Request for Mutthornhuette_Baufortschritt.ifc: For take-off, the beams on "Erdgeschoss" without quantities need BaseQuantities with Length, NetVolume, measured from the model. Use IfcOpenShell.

First a look at what the model holds.

```python
import ifcopenshell
import ifcopenshell.util.element
import ifcopenshell.util.unit

model = ifcopenshell.open("Mutthornhuette_Baufortschritt.ifc")
print(model.schema)
for unit_type in ("LENGTHUNIT", "AREAUNIT", "VOLUMEUNIT"):
    print(unit_type, ifcopenshell.util.unit.calculate_unit_scale(model, unit_type))
storey = next(s for s in model.by_type("IfcBuildingStorey") if s.Name == "Erdgeschoss")
beams = [e for e in ifcopenshell.util.element.get_decomposition(storey) if e.is_a("IfcBeam")]
for e in sorted(beams, key=lambda e: e.id()):
    print(e.id(), e.is_a(), e.Name, list(ifcopenshell.util.element.get_psets(e, qtos_only=True)), sep=" | ")
```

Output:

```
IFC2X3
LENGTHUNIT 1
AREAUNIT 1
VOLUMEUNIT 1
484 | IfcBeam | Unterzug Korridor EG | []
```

```python
import ifcopenshell
import ifcopenshell.api.pset
import ifcopenshell.geom
import ifcopenshell.util.element
import ifcopenshell.util.shape
import ifcopenshell.util.unit

model = ifcopenshell.open("Mutthornhuette_Baufortschritt.ifc")
unit_scale = ifcopenshell.util.unit.calculate_unit_scale(model)
volume_scale = ifcopenshell.util.unit.calculate_unit_scale(model, "VOLUMEUNIT")
settings = ifcopenshell.geom.settings()

storey = next(s for s in model.by_type("IfcBuildingStorey") if s.Name == "Erdgeschoss")
beams = [e for e in ifcopenshell.util.element.get_decomposition(storey) if e.is_a("IfcBeam")]

for e in sorted(beams, key=lambda e: e.id()):
    if ifcopenshell.util.element.get_psets(e, qtos_only=True, should_inherit=False):
        continue
    # Geometry comes back in metres, in the element's own axes.
    shape = ifcopenshell.geom.create_shape(settings, e)
    values = {
        "Length": ifcopenshell.util.shape.get_max_xyz(shape.geometry) / unit_scale,
        "NetVolume": ifcopenshell.util.shape.get_volume(shape.geometry) / volume_scale,
    }
    qto = ifcopenshell.api.pset.add_qto(model, product=e, name="BaseQuantities")
    ifcopenshell.api.pset.edit_qto(model, qto=qto, properties=values)
    print(e.id(), {k: round(v, 3) for k, v in values.items()})

model.write("Mutthornhuette_Baufortschritt_v2.ifc")
```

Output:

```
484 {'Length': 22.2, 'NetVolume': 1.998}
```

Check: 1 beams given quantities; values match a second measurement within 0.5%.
